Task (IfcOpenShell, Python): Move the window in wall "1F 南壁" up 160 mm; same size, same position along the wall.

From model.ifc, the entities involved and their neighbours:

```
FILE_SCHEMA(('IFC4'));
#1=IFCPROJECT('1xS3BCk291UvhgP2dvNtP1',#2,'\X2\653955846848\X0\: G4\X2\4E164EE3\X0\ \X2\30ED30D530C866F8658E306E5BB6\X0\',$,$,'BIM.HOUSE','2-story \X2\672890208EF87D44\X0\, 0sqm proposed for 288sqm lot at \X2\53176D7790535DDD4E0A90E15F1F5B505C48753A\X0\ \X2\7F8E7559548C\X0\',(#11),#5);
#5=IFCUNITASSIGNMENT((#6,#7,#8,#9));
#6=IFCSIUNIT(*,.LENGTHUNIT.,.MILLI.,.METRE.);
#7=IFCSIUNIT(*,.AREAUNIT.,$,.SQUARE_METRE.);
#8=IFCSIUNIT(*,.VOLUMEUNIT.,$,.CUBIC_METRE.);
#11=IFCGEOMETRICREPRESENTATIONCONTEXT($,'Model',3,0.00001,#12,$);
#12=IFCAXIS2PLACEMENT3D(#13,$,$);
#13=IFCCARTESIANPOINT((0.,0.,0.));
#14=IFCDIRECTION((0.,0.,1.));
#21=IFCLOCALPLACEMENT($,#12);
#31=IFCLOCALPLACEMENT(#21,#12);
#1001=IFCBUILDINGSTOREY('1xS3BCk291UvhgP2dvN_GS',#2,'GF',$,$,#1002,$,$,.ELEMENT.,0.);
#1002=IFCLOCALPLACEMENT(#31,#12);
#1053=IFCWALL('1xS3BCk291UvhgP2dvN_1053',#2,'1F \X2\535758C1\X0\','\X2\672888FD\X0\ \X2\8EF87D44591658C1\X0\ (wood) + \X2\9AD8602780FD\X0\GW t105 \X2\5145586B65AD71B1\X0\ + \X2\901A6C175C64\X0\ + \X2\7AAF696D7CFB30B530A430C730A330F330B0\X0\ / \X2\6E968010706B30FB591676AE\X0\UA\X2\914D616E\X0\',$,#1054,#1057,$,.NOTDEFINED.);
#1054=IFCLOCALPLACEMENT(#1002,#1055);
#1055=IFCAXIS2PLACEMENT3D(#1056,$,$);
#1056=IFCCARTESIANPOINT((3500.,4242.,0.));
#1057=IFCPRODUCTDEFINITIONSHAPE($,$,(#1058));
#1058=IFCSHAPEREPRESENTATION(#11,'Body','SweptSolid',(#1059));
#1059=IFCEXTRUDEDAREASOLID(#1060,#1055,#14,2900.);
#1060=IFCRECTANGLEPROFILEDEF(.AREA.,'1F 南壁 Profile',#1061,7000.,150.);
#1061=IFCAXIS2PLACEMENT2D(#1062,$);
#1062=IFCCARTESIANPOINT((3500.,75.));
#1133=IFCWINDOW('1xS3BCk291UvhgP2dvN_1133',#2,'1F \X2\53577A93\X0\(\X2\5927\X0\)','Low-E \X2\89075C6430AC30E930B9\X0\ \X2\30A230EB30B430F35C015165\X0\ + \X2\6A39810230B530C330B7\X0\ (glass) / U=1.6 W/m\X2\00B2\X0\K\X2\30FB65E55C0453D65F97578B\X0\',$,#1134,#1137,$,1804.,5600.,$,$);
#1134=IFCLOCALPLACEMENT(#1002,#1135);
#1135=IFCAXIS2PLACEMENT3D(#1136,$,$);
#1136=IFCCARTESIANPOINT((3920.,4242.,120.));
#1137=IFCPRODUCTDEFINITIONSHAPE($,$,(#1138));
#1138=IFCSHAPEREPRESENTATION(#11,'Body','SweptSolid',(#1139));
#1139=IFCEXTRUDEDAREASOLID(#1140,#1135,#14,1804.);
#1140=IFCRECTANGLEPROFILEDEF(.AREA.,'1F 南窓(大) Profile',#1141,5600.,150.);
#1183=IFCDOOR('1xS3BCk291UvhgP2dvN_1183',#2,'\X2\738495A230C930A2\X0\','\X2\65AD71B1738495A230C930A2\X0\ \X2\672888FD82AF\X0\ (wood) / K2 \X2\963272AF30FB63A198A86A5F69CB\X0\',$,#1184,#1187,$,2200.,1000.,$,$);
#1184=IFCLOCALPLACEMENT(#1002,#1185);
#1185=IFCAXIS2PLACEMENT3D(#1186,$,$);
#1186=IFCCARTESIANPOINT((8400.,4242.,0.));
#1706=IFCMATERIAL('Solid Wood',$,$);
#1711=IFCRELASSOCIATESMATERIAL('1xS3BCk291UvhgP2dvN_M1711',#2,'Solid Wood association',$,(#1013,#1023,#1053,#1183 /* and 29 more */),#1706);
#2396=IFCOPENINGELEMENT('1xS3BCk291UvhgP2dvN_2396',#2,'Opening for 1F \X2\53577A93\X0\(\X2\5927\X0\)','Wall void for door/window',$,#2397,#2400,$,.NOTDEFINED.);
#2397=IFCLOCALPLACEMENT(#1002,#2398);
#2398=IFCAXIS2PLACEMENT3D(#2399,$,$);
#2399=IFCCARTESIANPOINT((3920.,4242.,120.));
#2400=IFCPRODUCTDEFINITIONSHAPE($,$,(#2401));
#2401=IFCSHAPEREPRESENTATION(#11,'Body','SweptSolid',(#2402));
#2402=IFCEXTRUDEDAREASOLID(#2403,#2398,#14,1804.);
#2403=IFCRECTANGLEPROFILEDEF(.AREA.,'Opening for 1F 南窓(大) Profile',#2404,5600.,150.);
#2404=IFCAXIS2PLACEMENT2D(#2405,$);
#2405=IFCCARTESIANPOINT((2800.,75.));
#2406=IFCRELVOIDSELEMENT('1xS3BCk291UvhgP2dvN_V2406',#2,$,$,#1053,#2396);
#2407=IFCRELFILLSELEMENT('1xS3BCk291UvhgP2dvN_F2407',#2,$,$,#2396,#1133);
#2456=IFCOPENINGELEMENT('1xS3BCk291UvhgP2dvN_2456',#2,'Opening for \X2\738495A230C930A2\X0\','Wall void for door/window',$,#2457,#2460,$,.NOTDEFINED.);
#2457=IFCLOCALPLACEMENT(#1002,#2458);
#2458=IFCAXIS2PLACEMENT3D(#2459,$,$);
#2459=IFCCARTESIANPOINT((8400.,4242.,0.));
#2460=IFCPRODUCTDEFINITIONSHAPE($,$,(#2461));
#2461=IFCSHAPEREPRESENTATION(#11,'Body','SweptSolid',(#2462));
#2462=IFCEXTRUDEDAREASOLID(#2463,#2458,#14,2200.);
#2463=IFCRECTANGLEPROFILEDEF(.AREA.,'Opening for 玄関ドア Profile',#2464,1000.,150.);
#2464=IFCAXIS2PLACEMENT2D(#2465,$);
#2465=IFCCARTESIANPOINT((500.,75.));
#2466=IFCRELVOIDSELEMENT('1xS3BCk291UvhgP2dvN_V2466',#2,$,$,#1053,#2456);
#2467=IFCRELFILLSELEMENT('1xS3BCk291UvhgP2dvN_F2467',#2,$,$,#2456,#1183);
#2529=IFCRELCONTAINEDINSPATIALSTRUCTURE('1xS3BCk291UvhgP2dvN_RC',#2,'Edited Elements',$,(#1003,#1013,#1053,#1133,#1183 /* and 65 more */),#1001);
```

```python
import numpy as np
import ifcopenshell
import ifcopenshell.api.geometry
import ifcopenshell.util.placement
import ifcopenshell.util.unit

model = ifcopenshell.open("model.ifc")
unit_scale = ifcopenshell.util.unit.calculate_unit_scale(model)

window = model.by_guid("1xS3BCk291UvhgP2dvN_1133")
opening = window.FillsVoids[0].RelatingOpeningElement
dz = 160.0

shift = np.array([0.0, 0.0, dz])
# The window is not placed relative to its opening, so move both.
for product in (opening, window):
    matrix = ifcopenshell.util.placement.get_local_placement(product.ObjectPlacement)
    matrix[:3, 3] += shift
    ifcopenshell.api.geometry.edit_object_placement(model, product=product, matrix=matrix, is_si=False)

print(f"moved by {dz * unit_scale:+.3f} m")

model.write("model_rev.ifc")
```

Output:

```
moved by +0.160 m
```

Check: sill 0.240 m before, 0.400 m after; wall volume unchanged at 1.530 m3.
